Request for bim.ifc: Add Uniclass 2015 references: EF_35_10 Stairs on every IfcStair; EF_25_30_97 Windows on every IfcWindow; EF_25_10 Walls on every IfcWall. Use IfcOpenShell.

First a look at what the model holds.

```python
import ifcopenshell

model = ifcopenshell.open("bim.ifc")
print(model.schema)
print("classifications:", [c.Name for c in model.by_type("IfcClassification")])
for ifc_class in ("IfcDoor", "IfcRoof", "IfcStair", "IfcWall", "IfcWindow"):
    print(ifc_class, len(model.by_type(ifc_class)))
```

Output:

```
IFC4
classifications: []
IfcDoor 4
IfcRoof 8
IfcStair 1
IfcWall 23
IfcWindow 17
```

```python
import ifcopenshell
import ifcopenshell.api.classification

model = ifcopenshell.open("bim.ifc")

system = ifcopenshell.api.classification.add_classification(model, classification="Uniclass 2015")

codes = {
    "IfcStair": ("EF_35_10", "Stairs"),
    "IfcWindow": ("EF_25_30_97", "Windows"),
    "IfcWall": ("EF_25_10", "Walls"),
}
for ifc_class, (code, name) in codes.items():
    products = model.by_type(ifc_class)
    ifcopenshell.api.classification.add_reference(
        model, products=products, classification=system, identification=code, name=name
    )
    print(code, len(products))

model.write("bim_edited.ifc")
```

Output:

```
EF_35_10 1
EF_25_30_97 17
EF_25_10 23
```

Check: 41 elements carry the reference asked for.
